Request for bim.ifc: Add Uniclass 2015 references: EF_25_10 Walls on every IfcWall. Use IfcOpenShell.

First a look at what the model holds.

```python
import ifcopenshell

model = ifcopenshell.open("bim.ifc")
print(model.schema)
print("classifications:", [c.Name for c in model.by_type("IfcClassification")])
for ifc_class in ("IfcDoor", "IfcRoof", "IfcStair", "IfcWall", "IfcWindow"):
    print(ifc_class, len(model.by_type(ifc_class)))
```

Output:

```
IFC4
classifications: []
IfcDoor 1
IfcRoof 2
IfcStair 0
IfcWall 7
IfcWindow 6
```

```python
import ifcopenshell
import ifcopenshell.api.classification

model = ifcopenshell.open("bim.ifc")

system = ifcopenshell.api.classification.add_classification(model, classification="Uniclass 2015")

codes = {
    "IfcWall": ("EF_25_10", "Walls"),
}
for ifc_class, (code, name) in codes.items():
    products = model.by_type(ifc_class)
    ifcopenshell.api.classification.add_reference(
        model, products=products, classification=system, identification=code, name=name
    )
    print(code, len(products))

model.write("bim_updated.ifc")
```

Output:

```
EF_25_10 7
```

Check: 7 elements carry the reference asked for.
